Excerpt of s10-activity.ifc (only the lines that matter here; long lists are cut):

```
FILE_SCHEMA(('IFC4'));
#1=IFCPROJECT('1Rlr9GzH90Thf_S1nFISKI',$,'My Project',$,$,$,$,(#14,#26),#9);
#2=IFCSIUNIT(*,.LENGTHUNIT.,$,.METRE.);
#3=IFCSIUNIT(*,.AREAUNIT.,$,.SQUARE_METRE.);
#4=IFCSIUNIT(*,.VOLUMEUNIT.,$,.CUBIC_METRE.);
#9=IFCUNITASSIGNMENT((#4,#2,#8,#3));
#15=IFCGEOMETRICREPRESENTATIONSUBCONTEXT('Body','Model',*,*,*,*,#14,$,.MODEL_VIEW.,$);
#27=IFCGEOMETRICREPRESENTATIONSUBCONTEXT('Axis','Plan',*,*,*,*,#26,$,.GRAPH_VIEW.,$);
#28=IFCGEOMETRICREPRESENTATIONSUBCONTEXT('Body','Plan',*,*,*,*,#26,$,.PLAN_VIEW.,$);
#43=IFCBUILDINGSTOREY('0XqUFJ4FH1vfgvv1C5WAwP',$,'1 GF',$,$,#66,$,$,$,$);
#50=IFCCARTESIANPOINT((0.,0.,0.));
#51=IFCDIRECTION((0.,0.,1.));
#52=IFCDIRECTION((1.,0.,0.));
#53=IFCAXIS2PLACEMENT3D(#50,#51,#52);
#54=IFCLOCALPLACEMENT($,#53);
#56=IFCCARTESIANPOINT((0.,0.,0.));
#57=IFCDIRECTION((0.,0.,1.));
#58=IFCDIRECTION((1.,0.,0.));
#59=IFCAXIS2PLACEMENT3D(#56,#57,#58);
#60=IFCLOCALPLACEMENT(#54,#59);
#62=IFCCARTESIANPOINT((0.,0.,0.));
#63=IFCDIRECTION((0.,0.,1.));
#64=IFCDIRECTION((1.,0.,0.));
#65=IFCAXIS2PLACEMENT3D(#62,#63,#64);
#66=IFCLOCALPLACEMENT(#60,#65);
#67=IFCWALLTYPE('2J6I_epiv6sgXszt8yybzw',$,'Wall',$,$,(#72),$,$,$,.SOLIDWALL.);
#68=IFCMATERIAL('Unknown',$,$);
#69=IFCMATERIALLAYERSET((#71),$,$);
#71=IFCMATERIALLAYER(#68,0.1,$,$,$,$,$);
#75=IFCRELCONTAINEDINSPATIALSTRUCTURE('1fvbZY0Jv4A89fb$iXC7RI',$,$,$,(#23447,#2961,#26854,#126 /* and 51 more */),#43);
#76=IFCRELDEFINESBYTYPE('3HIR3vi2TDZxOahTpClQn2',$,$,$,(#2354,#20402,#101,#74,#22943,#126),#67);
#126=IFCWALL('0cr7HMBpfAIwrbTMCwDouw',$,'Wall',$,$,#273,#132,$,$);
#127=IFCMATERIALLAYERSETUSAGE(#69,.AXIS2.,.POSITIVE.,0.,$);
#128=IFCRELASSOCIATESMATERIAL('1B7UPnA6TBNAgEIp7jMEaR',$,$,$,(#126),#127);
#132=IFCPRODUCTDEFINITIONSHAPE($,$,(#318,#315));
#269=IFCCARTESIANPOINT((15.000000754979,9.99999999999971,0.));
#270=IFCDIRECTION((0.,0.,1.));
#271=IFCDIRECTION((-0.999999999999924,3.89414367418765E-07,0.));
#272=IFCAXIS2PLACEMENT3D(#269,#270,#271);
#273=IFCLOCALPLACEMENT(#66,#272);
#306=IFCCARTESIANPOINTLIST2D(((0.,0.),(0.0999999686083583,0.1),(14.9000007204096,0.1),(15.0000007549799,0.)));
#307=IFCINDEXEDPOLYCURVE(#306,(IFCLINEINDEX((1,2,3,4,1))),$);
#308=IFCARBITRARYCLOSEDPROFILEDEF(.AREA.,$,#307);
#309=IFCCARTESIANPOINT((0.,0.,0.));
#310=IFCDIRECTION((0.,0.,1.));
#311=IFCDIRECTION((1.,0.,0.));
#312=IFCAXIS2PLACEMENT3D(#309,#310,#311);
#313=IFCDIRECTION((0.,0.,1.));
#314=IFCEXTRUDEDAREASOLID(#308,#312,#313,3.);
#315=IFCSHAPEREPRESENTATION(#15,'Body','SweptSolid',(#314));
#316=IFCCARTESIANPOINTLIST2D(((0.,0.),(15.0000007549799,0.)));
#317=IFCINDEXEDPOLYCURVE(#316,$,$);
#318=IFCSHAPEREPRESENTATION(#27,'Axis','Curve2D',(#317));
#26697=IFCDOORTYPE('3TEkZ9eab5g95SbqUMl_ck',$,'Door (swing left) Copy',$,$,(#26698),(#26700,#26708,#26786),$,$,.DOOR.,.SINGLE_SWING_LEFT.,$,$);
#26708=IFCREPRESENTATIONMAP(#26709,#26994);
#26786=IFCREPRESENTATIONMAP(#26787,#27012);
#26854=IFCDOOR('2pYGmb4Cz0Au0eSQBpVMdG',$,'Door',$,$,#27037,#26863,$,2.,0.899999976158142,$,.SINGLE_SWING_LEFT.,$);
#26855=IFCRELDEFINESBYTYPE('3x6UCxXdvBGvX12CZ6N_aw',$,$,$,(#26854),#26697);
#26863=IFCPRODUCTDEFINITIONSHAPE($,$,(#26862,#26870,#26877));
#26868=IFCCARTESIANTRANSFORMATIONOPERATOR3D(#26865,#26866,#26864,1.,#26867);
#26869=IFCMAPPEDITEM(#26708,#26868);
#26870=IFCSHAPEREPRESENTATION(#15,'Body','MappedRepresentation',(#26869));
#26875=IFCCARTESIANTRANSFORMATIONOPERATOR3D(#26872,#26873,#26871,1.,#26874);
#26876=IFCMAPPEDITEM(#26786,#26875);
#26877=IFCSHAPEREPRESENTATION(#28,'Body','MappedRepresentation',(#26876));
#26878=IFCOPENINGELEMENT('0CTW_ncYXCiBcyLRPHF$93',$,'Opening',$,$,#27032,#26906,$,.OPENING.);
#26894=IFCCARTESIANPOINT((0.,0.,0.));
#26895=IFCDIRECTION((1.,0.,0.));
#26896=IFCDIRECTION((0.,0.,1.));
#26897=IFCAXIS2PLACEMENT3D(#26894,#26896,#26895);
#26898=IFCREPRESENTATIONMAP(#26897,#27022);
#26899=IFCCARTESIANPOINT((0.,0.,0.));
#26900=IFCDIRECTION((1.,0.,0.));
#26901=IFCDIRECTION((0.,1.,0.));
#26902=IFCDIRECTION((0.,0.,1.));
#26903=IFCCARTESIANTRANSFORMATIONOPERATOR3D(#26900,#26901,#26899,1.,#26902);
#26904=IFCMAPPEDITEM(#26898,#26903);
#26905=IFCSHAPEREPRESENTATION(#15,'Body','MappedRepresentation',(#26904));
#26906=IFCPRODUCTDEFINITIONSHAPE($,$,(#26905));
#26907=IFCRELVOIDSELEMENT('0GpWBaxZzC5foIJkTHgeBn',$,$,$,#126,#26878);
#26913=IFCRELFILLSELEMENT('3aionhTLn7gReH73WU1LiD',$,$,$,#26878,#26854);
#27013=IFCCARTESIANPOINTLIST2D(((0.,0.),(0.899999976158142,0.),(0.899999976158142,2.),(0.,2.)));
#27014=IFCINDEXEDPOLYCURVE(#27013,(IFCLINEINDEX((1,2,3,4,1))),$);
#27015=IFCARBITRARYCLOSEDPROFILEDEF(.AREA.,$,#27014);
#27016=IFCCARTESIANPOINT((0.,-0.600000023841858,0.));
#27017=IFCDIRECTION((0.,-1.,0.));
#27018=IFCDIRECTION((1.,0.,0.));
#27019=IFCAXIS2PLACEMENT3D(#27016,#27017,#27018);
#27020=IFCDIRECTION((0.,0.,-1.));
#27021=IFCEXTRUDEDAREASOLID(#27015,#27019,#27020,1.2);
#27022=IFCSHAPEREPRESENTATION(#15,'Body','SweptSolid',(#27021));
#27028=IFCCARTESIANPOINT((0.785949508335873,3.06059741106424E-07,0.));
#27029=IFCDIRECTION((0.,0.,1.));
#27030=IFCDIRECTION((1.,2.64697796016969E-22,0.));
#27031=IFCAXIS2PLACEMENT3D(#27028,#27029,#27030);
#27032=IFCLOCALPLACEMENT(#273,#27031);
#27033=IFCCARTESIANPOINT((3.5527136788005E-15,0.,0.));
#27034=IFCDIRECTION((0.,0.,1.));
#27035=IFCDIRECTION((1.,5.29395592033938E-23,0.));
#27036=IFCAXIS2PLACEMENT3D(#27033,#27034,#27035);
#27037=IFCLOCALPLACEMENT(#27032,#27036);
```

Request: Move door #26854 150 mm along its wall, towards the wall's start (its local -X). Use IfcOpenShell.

```python
import ifcopenshell
import ifcopenshell.api.geometry
import ifcopenshell.util.placement
import ifcopenshell.util.unit

model = ifcopenshell.open("s10-activity.ifc")
unit_scale = ifcopenshell.util.unit.calculate_unit_scale(model)

door = model.by_id(26854)
opening = door.FillsVoids[0].RelatingOpeningElement
wall = opening.VoidsElements[0].RelatingBuildingElement

wall_matrix = ifcopenshell.util.placement.get_local_placement(wall.ObjectPlacement)
shift = wall_matrix[:3, 0] * -0.15 / unit_scale
before = ifcopenshell.util.placement.get_local_placement(door.ObjectPlacement)[:3, 3].copy()

# The door is placed relative to its opening, so it follows when the opening moves.
matrix = ifcopenshell.util.placement.get_local_placement(opening.ObjectPlacement)
matrix[:3, 3] += shift
ifcopenshell.api.geometry.edit_object_placement(
    model, product=opening, matrix=matrix, is_si=False, should_transform_children=True
)

after = ifcopenshell.util.placement.get_local_placement(door.ObjectPlacement)[:3, 3]
print("door moved by", (after - before).round(3) + 0.0)

model.write("s10-activity_edited.ifc")
```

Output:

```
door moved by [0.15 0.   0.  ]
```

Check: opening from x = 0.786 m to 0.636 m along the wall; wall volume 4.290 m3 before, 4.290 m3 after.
